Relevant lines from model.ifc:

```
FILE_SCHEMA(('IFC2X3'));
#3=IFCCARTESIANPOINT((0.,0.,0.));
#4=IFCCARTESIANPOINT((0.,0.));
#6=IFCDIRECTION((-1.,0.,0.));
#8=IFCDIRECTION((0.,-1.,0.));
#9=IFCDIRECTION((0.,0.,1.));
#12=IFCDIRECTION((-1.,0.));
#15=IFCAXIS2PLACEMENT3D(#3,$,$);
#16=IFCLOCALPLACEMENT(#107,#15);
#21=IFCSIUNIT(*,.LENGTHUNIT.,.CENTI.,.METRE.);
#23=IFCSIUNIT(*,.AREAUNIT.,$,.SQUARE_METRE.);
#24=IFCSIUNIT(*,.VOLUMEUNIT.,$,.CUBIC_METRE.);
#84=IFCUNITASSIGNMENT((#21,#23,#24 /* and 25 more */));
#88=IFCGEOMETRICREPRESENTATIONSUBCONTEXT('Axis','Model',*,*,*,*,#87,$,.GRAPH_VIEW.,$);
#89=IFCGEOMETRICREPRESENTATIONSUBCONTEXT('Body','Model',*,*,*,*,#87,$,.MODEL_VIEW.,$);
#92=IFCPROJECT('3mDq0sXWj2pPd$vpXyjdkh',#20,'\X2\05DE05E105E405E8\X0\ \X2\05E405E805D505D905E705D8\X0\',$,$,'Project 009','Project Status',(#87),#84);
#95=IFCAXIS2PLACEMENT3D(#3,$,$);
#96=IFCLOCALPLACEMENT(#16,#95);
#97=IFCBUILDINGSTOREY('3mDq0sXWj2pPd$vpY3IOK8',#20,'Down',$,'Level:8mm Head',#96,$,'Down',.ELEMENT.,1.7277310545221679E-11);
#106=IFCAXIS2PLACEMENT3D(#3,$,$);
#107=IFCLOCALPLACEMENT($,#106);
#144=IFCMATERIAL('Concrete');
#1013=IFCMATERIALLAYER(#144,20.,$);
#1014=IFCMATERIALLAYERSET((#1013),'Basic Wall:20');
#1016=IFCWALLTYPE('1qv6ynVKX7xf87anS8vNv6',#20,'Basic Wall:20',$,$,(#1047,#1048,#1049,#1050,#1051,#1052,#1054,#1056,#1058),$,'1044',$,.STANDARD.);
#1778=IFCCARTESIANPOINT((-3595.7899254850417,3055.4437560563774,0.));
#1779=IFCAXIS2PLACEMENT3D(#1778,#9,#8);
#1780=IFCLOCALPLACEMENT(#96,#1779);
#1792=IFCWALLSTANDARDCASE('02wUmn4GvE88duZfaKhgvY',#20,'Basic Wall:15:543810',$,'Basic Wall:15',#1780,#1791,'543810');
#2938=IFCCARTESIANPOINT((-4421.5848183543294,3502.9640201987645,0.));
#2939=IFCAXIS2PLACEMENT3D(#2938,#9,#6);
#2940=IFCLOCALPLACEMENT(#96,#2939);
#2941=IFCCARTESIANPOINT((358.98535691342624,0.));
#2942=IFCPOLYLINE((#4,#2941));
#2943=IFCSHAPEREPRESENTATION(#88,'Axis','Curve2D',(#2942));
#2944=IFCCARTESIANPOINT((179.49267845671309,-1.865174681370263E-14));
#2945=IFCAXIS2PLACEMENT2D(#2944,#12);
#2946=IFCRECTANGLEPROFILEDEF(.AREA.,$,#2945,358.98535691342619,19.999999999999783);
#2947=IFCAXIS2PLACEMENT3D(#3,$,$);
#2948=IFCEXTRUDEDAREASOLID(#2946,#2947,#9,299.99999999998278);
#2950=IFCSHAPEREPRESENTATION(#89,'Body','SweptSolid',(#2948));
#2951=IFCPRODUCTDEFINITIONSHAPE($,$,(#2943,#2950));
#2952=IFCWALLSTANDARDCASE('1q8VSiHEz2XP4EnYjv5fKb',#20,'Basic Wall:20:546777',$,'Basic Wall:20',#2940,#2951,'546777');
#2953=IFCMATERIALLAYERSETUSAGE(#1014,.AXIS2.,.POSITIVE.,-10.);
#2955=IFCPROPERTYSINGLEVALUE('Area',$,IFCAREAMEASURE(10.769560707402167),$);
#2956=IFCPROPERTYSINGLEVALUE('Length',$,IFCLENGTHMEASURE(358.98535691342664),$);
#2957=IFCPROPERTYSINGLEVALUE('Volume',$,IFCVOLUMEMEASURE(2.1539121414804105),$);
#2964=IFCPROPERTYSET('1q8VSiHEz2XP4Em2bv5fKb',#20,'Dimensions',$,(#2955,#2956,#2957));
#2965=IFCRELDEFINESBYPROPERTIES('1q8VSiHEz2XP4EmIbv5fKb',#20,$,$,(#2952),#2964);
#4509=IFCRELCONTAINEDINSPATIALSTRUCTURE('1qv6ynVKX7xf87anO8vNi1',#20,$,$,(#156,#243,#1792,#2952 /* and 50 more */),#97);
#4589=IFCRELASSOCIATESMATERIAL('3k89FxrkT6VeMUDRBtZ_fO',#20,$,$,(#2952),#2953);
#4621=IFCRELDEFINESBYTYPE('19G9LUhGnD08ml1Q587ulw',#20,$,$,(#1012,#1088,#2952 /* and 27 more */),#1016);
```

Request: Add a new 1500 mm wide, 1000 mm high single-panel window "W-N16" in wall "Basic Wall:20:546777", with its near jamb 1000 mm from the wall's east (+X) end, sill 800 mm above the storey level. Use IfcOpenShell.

```python
import numpy as np
import ifcopenshell
import ifcopenshell.api.feature
import ifcopenshell.api.geometry
import ifcopenshell.api.pset
import ifcopenshell.api.root
import ifcopenshell.api.spatial
import ifcopenshell.api.type
import ifcopenshell.geom
import ifcopenshell.util.element
import ifcopenshell.util.placement
import ifcopenshell.util.representation
import ifcopenshell.util.shape
import ifcopenshell.util.unit

model = ifcopenshell.open("model.ifc")
unit_scale = ifcopenshell.util.unit.calculate_unit_scale(model)
area_scale = ifcopenshell.util.unit.calculate_unit_scale(model, "AREAUNIT")
volume_scale = ifcopenshell.util.unit.calculate_unit_scale(model, "VOLUMEUNIT")
settings = ifcopenshell.geom.settings()


def volume(element):
    """Net volume in cubic metres, openings subtracted."""
    shape = ifcopenshell.geom.create_shape(settings, element)
    return ifcopenshell.util.shape.get_volume(shape.geometry)


wall = model.by_guid("1q8VSiHEz2XP4EnYjv5fKb")
storey = ifcopenshell.util.element.get_container(wall, ifc_class="IfcBuildingStorey")
context = ifcopenshell.util.representation.get_context(model, "Model", "Body", "MODEL_VIEW")
before = volume(wall)

width, height, from_end, sill = 1.5, 1, 1, 0.8  # metres

# The wall runs along its own X axis, and the end named is its -X end.
wall_shape = ifcopenshell.geom.create_shape(settings, wall)
x, y, z = ifcopenshell.util.shape.get_vertices(wall_shape.geometry).T
start = x.min() + from_end
face, thickness = float(y.min()), float(y.max() - y.min())
wall_matrix = ifcopenshell.util.placement.get_local_placement(wall.ObjectPlacement)
level = ifcopenshell.util.placement.get_local_placement(storey.ObjectPlacement)[2, 3]


def in_wall(x, y):
    """Placement at x, y metres in the wall's axes, at sill height."""
    matrix = wall_matrix.copy()
    matrix[:, 3] = wall_matrix @ np.array([x / unit_scale, y / unit_scale, 0.0, 1.0])
    matrix[2, 3] = level + sill / unit_scale
    return matrix


# Opening: a box that overshoots both wall faces by 50 mm.
opening = ifcopenshell.api.root.create_entity(model, ifc_class="IfcOpeningElement")
box = ifcopenshell.api.geometry.add_wall_representation(
    model, context=context, length=width, height=height, thickness=thickness + 0.1
)
ifcopenshell.api.geometry.assign_representation(model, product=opening, representation=box)
ifcopenshell.api.geometry.edit_object_placement(model, product=opening, matrix=in_wall(start, face - 0.05), is_si=False)
ifcopenshell.api.feature.add_feature(model, feature=opening, element=wall)

window = ifcopenshell.api.root.create_entity(model, ifc_class="IfcWindow", name="W-N16")
window.OverallWidth, window.OverallHeight = width / unit_scale, height / unit_scale
body = ifcopenshell.api.geometry.add_window_representation(
    model,
    context=context,
    overall_width=window.OverallWidth,
    overall_height=window.OverallHeight,
    partition_type="SINGLE_PANEL",
)
ifcopenshell.api.geometry.assign_representation(model, product=window, representation=body)
ifcopenshell.api.spatial.assign_container(model, products=[window], relating_structure=storey)
fills = ifcopenshell.api.feature.add_filling(model, opening=opening, element=window)
fills.OwnerHistory = window.OwnerHistory  # required in IFC2X3

# IFC2X3 keeps the operation on the window style.
style = ifcopenshell.api.root.create_entity(model, ifc_class="IfcWindowStyle", name="W-N16")
style.OperationType, style.ConstructionType = "SINGLE_PANEL", "NOTDEFINED"
style.ParameterTakesPrecedence = style.Sizeable = False
ifcopenshell.api.type.assign_type(model, related_objects=[window], relating_type=style)

# Centre the window in the wall's thickness.
ifcopenshell.api.geometry.edit_object_placement(model, product=window, matrix=in_wall(start, face), is_si=False)
window_shape = ifcopenshell.geom.create_shape(settings, window)
depth = ifcopenshell.util.shape.get_vertices(window_shape.geometry)[:, 1]
offset = face + thickness / 2 - (depth.min() + depth.max()) / 2
ifcopenshell.api.geometry.edit_object_placement(model, product=window, matrix=in_wall(start, offset), is_si=False)

after = volume(wall)

# Update the wall's stored quantities.
pset = model.by_id(ifcopenshell.util.element.get_pset(wall, "Dimensions", should_inherit=False)["id"])
ifcopenshell.api.pset.edit_pset(model, pset=pset, properties={
    "Area": model.create_entity("IfcAreaMeasure", after / thickness / area_scale),
    "Volume": model.create_entity("IfcVolumeMeasure", after / volume_scale),
})

print(f"wall volume {before:.3f} -> {after:.3f} m3")

model.write("model_v2.ifc")
```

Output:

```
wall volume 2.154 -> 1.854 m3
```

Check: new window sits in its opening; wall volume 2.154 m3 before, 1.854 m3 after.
